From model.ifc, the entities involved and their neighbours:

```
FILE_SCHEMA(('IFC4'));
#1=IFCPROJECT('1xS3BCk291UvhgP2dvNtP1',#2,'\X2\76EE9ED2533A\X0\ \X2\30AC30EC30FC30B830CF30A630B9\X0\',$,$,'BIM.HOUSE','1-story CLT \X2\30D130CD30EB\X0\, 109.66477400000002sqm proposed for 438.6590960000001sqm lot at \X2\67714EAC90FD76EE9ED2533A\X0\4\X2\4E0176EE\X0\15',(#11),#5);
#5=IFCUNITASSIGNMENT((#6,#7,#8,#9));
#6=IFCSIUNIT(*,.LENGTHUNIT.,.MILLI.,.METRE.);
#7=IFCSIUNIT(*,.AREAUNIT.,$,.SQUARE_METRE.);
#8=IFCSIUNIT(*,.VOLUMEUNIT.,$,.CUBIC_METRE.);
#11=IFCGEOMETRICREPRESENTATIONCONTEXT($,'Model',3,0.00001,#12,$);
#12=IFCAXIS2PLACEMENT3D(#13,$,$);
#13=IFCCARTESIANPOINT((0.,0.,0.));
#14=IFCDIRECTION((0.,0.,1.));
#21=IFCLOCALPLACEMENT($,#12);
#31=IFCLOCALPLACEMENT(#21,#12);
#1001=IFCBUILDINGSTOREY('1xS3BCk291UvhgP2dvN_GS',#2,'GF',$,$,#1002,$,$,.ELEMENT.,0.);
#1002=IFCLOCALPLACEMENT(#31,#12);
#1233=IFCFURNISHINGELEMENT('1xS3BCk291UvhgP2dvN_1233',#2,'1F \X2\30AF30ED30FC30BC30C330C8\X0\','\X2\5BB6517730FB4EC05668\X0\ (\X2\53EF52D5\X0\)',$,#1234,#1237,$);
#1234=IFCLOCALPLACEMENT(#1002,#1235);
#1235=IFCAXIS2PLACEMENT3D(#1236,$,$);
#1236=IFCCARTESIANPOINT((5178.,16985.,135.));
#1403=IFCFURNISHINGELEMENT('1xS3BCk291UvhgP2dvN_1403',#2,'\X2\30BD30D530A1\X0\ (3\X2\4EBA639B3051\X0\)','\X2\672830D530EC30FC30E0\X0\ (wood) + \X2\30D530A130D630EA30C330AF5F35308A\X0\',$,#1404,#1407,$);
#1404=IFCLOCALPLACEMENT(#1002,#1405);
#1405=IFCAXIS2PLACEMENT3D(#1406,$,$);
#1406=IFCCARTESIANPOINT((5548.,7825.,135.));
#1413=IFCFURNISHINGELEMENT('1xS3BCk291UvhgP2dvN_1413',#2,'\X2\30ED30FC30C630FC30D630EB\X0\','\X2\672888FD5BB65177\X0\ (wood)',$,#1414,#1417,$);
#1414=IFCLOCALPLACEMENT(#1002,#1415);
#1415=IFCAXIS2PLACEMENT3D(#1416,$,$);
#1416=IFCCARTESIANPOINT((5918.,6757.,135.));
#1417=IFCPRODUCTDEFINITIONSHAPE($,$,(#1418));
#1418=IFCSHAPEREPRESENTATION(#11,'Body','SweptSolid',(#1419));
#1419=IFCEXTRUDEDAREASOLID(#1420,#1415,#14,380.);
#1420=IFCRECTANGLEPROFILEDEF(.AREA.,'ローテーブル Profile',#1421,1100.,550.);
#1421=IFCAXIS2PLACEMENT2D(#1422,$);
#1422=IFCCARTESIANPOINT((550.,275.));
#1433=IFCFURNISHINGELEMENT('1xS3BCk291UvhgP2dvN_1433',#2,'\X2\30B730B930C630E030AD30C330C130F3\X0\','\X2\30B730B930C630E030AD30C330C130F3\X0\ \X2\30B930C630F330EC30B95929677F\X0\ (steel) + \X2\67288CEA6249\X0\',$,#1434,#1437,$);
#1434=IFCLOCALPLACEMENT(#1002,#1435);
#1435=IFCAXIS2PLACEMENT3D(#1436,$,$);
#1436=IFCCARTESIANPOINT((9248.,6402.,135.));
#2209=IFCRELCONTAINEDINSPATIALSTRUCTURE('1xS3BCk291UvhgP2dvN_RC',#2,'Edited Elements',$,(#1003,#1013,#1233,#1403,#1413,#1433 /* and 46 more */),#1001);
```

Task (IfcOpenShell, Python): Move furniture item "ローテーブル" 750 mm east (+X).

```python
import ifcopenshell
import ifcopenshell.api.geometry
import ifcopenshell.util.placement
import ifcopenshell.util.unit

model = ifcopenshell.open("model.ifc")
unit_scale = ifcopenshell.util.unit.calculate_unit_scale(model)

item = model.by_id(1413)
matrix = ifcopenshell.util.placement.get_local_placement(item.ObjectPlacement)
matrix[0, 3] += 0.75 / unit_scale
ifcopenshell.api.geometry.edit_object_placement(model, product=item, matrix=matrix, is_si=False)

print(ifcopenshell.util.placement.get_local_placement(item.ObjectPlacement).round(3) + 0.0)

model.write("model-out.ifc")
```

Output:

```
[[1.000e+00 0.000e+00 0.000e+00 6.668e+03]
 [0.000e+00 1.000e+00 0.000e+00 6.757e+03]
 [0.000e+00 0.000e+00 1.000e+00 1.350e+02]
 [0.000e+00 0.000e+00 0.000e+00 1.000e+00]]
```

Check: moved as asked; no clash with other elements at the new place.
